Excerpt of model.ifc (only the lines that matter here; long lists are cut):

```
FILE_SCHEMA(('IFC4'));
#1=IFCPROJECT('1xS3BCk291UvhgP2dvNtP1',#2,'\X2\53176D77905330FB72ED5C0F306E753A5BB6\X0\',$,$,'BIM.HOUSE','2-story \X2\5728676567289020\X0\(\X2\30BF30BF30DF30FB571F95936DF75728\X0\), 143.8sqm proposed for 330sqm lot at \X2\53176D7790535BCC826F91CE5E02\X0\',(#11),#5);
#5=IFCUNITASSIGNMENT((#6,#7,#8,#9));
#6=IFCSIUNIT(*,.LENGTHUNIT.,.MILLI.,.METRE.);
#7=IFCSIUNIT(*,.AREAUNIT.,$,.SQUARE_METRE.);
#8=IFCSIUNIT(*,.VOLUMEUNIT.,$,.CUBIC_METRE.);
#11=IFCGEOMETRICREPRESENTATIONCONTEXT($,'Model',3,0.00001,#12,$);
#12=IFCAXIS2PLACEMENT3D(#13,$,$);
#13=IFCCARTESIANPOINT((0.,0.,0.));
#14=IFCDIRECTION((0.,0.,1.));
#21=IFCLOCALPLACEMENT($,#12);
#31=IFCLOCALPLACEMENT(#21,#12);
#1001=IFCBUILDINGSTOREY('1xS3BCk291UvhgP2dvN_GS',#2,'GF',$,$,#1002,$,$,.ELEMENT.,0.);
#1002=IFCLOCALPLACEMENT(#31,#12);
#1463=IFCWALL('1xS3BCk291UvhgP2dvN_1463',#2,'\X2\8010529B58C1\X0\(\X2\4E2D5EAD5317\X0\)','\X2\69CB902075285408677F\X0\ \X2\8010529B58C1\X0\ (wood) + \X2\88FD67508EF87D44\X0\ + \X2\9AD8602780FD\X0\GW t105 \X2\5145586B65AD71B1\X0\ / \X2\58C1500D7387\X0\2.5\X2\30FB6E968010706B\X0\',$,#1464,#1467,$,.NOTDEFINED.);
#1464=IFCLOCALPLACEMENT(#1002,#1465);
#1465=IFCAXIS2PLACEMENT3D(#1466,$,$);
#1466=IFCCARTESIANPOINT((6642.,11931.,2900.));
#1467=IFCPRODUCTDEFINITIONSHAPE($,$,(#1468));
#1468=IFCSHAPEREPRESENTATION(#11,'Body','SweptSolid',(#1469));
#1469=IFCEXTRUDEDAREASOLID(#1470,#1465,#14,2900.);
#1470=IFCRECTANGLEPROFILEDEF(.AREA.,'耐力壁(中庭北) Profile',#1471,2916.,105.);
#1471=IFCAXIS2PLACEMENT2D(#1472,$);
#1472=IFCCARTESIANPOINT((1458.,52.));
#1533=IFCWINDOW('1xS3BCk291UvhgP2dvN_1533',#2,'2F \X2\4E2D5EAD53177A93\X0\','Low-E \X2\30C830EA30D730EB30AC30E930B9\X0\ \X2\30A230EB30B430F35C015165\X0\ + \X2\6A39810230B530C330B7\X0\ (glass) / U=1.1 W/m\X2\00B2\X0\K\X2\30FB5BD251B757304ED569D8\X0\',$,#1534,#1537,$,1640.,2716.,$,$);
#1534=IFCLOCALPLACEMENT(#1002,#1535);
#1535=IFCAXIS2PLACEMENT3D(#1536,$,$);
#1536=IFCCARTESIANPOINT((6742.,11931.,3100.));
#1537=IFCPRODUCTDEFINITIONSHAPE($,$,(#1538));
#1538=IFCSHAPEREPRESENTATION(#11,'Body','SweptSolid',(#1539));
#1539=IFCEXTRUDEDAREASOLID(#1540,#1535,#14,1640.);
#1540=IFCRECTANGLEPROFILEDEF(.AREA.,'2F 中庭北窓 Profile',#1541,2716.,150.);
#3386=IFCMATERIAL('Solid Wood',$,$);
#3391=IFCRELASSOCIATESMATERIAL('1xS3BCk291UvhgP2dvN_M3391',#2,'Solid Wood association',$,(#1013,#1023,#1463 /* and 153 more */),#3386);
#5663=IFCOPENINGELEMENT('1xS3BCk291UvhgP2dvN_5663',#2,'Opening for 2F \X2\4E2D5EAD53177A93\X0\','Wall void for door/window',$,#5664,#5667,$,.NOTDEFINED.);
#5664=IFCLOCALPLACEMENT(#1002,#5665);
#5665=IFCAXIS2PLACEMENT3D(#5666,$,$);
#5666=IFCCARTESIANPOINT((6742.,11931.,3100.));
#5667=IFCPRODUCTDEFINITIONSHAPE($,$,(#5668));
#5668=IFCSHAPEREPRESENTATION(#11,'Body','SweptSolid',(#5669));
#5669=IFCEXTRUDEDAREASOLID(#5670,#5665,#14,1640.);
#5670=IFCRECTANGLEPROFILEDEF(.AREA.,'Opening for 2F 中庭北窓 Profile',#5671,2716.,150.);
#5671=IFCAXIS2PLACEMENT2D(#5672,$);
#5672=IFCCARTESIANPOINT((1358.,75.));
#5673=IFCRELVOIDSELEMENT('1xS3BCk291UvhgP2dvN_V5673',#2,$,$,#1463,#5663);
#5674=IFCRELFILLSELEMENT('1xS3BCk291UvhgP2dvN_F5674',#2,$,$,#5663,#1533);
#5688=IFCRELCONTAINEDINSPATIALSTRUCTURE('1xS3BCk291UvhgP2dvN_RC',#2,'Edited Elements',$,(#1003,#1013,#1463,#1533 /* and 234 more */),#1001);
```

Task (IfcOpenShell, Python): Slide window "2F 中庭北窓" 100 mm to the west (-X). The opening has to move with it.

```python
import ifcopenshell
import ifcopenshell.api.geometry
import ifcopenshell.util.placement
import ifcopenshell.util.unit

model = ifcopenshell.open("model.ifc")
unit_scale = ifcopenshell.util.unit.calculate_unit_scale(model)

window = model.by_id(1533)
opening = window.FillsVoids[0].RelatingOpeningElement
wall = opening.VoidsElements[0].RelatingBuildingElement

wall_matrix = ifcopenshell.util.placement.get_local_placement(wall.ObjectPlacement)
shift = wall_matrix[:3, 0] * -0.1 / unit_scale
before = ifcopenshell.util.placement.get_local_placement(window.ObjectPlacement)[:3, 3].copy()

# The window is not placed relative to its opening, so move both.
for product in (opening, window):
    matrix = ifcopenshell.util.placement.get_local_placement(product.ObjectPlacement)
    matrix[:3, 3] += shift
    ifcopenshell.api.geometry.edit_object_placement(model, product=product, matrix=matrix, is_si=False)

after = ifcopenshell.util.placement.get_local_placement(window.ObjectPlacement)[:3, 3]
print("window moved by", (after - before).round(3) + 0.0)

model.write("model_rev.ifc")
```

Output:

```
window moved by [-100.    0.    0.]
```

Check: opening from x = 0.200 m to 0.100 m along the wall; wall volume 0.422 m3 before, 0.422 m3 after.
